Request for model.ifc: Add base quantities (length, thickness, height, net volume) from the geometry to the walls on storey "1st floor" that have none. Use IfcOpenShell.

First a look at what the model holds.

```python
import ifcopenshell
import ifcopenshell.util.element
import ifcopenshell.util.unit

model = ifcopenshell.open("model.ifc")
print(model.schema)
for unit_type in ("LENGTHUNIT", "AREAUNIT", "VOLUMEUNIT"):
    print(unit_type, ifcopenshell.util.unit.calculate_unit_scale(model, unit_type))
storey = next(s for s in model.by_type("IfcBuildingStorey") if s.Name == "1st floor")
walls = [e for e in ifcopenshell.util.element.get_decomposition(storey) if e.is_a("IfcWall")]
for e in sorted(walls, key=lambda e: e.id()):
    print(e.id(), e.is_a(), e.Name, list(ifcopenshell.util.element.get_psets(e, qtos_only=True)), sep=" | ")
```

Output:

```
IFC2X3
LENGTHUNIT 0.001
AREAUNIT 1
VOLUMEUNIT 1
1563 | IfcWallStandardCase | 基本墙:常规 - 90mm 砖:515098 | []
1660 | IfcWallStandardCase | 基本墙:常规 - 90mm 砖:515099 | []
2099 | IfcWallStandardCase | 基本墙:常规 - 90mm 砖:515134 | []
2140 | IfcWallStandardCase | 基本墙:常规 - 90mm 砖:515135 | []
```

```python
import ifcopenshell
import ifcopenshell.api.pset
import ifcopenshell.geom
import ifcopenshell.util.element
import ifcopenshell.util.shape
import ifcopenshell.util.unit

model = ifcopenshell.open("model.ifc")
unit_scale = ifcopenshell.util.unit.calculate_unit_scale(model)
volume_scale = ifcopenshell.util.unit.calculate_unit_scale(model, "VOLUMEUNIT")
settings = ifcopenshell.geom.settings()

storey = next(s for s in model.by_type("IfcBuildingStorey") if s.Name == "1st floor")
walls = [e for e in ifcopenshell.util.element.get_decomposition(storey) if e.is_a("IfcWall")]

for e in sorted(walls, key=lambda e: e.id()):
    if ifcopenshell.util.element.get_psets(e, qtos_only=True, should_inherit=False):
        continue
    # Geometry comes back in metres, in the element's own axes.
    shape = ifcopenshell.geom.create_shape(settings, e)
    values = {
        "Length": ifcopenshell.util.shape.get_x(shape.geometry) / unit_scale,
        "Width": ifcopenshell.util.shape.get_y(shape.geometry) / unit_scale,
        "Height": ifcopenshell.util.shape.get_z(shape.geometry) / unit_scale,
        "NetVolume": ifcopenshell.util.shape.get_volume(shape.geometry) / volume_scale,
    }
    qto = ifcopenshell.api.pset.add_qto(model, product=e, name="BaseQuantities")
    ifcopenshell.api.pset.edit_qto(model, qto=qto, properties=values)
    print(e.id(), {k: round(v, 3) for k, v in values.items()})

model.write("model_updated.ifc")
```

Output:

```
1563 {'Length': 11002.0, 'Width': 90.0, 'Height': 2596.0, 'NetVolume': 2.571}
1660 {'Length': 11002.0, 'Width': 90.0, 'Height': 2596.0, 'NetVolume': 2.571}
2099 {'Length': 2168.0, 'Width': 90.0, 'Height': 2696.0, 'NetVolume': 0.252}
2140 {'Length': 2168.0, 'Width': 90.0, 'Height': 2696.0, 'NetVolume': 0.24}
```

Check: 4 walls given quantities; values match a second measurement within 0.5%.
